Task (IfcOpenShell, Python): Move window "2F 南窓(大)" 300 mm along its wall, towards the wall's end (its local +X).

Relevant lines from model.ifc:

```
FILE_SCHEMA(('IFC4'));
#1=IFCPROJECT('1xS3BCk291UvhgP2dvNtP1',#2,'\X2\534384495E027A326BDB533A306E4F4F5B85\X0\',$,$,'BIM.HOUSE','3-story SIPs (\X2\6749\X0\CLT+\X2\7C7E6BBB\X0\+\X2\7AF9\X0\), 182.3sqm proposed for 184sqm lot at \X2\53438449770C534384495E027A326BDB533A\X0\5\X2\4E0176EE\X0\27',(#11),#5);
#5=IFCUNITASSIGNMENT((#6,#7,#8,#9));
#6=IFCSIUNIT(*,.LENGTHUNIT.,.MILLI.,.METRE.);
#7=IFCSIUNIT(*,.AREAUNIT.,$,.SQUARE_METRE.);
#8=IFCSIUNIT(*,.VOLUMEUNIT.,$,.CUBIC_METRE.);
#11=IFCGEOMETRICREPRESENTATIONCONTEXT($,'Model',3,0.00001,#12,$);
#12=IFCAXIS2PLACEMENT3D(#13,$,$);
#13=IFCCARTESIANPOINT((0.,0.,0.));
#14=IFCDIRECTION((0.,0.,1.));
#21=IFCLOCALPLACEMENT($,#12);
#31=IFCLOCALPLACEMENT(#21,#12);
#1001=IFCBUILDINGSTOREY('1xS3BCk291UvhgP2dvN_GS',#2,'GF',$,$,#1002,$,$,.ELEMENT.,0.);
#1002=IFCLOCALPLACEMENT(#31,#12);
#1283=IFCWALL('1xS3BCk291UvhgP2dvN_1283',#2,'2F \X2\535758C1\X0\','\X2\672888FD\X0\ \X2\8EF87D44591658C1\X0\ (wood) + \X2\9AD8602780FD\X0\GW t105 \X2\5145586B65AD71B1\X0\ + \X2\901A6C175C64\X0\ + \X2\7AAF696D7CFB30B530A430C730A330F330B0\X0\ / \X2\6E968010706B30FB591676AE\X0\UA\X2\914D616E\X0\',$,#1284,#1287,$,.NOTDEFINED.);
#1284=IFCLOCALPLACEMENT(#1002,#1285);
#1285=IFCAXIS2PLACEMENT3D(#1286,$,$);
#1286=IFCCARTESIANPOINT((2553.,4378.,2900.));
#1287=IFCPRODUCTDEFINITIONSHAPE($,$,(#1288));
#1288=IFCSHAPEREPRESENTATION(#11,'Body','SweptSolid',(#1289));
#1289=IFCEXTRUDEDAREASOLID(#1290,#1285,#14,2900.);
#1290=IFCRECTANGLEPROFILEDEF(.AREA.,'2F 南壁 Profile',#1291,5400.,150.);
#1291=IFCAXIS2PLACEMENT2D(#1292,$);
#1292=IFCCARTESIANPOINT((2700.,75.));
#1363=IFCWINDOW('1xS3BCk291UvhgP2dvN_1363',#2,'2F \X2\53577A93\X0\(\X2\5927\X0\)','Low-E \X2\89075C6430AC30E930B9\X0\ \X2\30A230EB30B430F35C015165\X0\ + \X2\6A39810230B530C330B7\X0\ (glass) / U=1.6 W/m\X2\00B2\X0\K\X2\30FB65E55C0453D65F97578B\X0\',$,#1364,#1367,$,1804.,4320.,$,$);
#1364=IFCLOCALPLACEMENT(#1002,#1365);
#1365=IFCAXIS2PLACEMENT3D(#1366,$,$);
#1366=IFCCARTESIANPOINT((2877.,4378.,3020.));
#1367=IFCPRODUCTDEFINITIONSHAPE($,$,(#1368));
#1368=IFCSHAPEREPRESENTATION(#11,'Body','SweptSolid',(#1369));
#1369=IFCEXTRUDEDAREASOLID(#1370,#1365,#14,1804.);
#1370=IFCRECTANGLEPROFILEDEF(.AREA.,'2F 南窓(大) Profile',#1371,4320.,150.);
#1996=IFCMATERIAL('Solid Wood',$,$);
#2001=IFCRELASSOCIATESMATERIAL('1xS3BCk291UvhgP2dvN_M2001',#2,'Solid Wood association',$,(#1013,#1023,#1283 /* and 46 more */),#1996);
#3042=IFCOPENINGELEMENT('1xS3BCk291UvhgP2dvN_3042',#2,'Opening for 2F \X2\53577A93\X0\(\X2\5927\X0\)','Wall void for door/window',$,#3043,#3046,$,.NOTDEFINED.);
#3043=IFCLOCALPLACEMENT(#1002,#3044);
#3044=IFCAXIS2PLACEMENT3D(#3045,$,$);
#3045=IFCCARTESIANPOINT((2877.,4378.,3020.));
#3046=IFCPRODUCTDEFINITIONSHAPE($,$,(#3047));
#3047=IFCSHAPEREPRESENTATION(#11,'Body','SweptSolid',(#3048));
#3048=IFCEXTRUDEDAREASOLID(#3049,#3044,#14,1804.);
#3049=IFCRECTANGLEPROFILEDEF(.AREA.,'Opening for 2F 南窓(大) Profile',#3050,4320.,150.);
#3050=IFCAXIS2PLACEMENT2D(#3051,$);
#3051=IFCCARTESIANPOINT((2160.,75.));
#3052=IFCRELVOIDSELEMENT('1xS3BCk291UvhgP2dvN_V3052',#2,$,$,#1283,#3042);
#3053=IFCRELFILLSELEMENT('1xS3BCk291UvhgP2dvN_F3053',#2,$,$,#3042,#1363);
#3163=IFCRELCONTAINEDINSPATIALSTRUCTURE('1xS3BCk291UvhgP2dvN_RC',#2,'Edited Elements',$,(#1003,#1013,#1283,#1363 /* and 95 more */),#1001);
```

```python
import ifcopenshell
import ifcopenshell.api.geometry
import ifcopenshell.util.placement
import ifcopenshell.util.unit

model = ifcopenshell.open("model.ifc")
unit_scale = ifcopenshell.util.unit.calculate_unit_scale(model)

window = model.by_guid("1xS3BCk291UvhgP2dvN_1363")
opening = window.FillsVoids[0].RelatingOpeningElement
wall = opening.VoidsElements[0].RelatingBuildingElement

wall_matrix = ifcopenshell.util.placement.get_local_placement(wall.ObjectPlacement)
shift = wall_matrix[:3, 0] * 0.3 / unit_scale
before = ifcopenshell.util.placement.get_local_placement(window.ObjectPlacement)[:3, 3].copy()

# The window is not placed relative to its opening, so move both.
for product in (opening, window):
    matrix = ifcopenshell.util.placement.get_local_placement(product.ObjectPlacement)
    matrix[:3, 3] += shift
    ifcopenshell.api.geometry.edit_object_placement(model, product=product, matrix=matrix, is_si=False)

after = ifcopenshell.util.placement.get_local_placement(window.ObjectPlacement)[:3, 3]
print("window moved by", (after - before).round(3) + 0.0)

model.write("model-out.ifc")
```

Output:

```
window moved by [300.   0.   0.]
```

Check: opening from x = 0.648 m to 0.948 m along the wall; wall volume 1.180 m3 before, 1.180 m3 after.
